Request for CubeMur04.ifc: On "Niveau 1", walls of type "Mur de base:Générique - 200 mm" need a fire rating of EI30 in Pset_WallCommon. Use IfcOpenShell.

First a look at what the model holds.

```python
import ifcopenshell
import ifcopenshell.util.element

model = ifcopenshell.open("CubeMur04.ifc")
print(model.schema)
storey = next(s for s in model.by_type("IfcBuildingStorey") if s.Name == "Niveau 1")
walls = [e for e in ifcopenshell.util.element.get_decomposition(storey) if e.is_a("IfcWall")]
seen = {}
for e in walls:
    element_type = ifcopenshell.util.element.get_type(e)
    key = (element_type.Name if element_type != e and element_type else None, ifcopenshell.util.element.get_pset(e, "Pset_WallCommon", "FireRating"))
    seen[key] = seen.get(key, 0) + 1
for (name, value), count in sorted(seen.items(), key=str):
    print(count, "x", name, "|", value)
```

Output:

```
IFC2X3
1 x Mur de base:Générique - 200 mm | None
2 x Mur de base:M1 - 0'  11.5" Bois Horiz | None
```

```python
import ifcopenshell
import ifcopenshell.api.pset
import ifcopenshell.util.element

model = ifcopenshell.open("CubeMur04.ifc")

storey = next(s for s in model.by_type("IfcBuildingStorey") if s.Name == "Niveau 1")
walls = [e for e in ifcopenshell.util.element.get_decomposition(storey) if e.is_a("IfcWall")]

count = 0
for e in walls:
    element_type = ifcopenshell.util.element.get_type(e)
    if element_type in (None, e) or element_type.Name != "Mur de base:Générique - 200 mm":
        continue
    # add_pset returns the element's existing set when there is one.
    pset = ifcopenshell.api.pset.add_pset(model, product=e, name="Pset_WallCommon")
    ifcopenshell.api.pset.edit_pset(model, pset=pset, properties={"FireRating": "EI30"})
    count += 1

print(count, "walls updated")

model.write("CubeMur04_v2.ifc")
```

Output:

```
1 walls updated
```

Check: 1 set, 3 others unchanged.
